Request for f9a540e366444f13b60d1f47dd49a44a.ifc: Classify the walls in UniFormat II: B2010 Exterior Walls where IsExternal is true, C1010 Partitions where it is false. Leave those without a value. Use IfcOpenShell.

First a look at what the model holds.

```python
import ifcopenshell
import ifcopenshell.util.element

model = ifcopenshell.open("f9a540e366444f13b60d1f47dd49a44a.ifc")
print(model.schema)
print("classifications:", [c.Name for c in model.by_type("IfcClassification")])
values = [ifcopenshell.util.element.get_pset(e, "Pset_WallCommon", "IsExternal") for e in model.by_type("IfcWall")]
for value in (True, False, None):
    print("IsExternal", value, values.count(value))
```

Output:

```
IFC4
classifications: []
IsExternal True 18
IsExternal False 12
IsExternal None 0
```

```python
import ifcopenshell
import ifcopenshell.api.classification
import ifcopenshell.util.element

model = ifcopenshell.open("f9a540e366444f13b60d1f47dd49a44a.ifc")

system = ifcopenshell.api.classification.add_classification(model, classification="UniFormat II")

walls = model.by_type("IfcWall")
external = {e: ifcopenshell.util.element.get_pset(e, "Pset_WallCommon", "IsExternal") for e in walls}
for flag, code, name in ((True, "B2010", "Exterior Walls"), (False, "C1010", "Partitions")):
    products = [e for e in walls if external[e] is flag]
    ifcopenshell.api.classification.add_reference(
        model, products=products, classification=system, identification=code, name=name
    )
    print(code, len(products))

model.write("f9a540e366444f13b60d1f47dd49a44a_rev.ifc")
```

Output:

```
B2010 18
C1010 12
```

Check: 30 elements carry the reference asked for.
